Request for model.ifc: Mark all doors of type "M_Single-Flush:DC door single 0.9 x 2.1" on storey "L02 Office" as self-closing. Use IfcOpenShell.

First a look at what the model holds.

```python
import ifcopenshell
import ifcopenshell.util.element

model = ifcopenshell.open("model.ifc")
print(model.schema)
storey = next(s for s in model.by_type("IfcBuildingStorey") if s.Name == "L02 Office")
doors = [e for e in ifcopenshell.util.element.get_decomposition(storey) if e.is_a("IfcDoor")]
seen = {}
for e in doors:
    element_type = ifcopenshell.util.element.get_type(e)
    key = (element_type.Name if element_type != e and element_type else None, ifcopenshell.util.element.get_pset(e, "Pset_DoorCommon", "SelfClosing"))
    seen[key] = seen.get(key, 0) + 1
for (name, value), count in sorted(seen.items(), key=str):
    print(count, "x", name, "|", value)
```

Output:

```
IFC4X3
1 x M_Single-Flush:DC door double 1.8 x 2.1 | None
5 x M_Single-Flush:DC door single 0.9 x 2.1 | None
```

```python
import ifcopenshell
import ifcopenshell.api.pset
import ifcopenshell.util.element

model = ifcopenshell.open("model.ifc")

storey = next(s for s in model.by_type("IfcBuildingStorey") if s.Name == "L02 Office")
doors = [e for e in ifcopenshell.util.element.get_decomposition(storey) if e.is_a("IfcDoor")]

count = 0
for e in doors:
    element_type = ifcopenshell.util.element.get_type(e)
    if element_type in (None, e) or element_type.Name != "M_Single-Flush:DC door single 0.9 x 2.1":
        continue
    # add_pset returns the element's existing set when there is one.
    pset = ifcopenshell.api.pset.add_pset(model, product=e, name="Pset_DoorCommon")
    ifcopenshell.api.pset.edit_pset(model, pset=pset, properties={"SelfClosing": True})
    count += 1

print(count, "doors updated")

model.write("model_updated.ifc")
```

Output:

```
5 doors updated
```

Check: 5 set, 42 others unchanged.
